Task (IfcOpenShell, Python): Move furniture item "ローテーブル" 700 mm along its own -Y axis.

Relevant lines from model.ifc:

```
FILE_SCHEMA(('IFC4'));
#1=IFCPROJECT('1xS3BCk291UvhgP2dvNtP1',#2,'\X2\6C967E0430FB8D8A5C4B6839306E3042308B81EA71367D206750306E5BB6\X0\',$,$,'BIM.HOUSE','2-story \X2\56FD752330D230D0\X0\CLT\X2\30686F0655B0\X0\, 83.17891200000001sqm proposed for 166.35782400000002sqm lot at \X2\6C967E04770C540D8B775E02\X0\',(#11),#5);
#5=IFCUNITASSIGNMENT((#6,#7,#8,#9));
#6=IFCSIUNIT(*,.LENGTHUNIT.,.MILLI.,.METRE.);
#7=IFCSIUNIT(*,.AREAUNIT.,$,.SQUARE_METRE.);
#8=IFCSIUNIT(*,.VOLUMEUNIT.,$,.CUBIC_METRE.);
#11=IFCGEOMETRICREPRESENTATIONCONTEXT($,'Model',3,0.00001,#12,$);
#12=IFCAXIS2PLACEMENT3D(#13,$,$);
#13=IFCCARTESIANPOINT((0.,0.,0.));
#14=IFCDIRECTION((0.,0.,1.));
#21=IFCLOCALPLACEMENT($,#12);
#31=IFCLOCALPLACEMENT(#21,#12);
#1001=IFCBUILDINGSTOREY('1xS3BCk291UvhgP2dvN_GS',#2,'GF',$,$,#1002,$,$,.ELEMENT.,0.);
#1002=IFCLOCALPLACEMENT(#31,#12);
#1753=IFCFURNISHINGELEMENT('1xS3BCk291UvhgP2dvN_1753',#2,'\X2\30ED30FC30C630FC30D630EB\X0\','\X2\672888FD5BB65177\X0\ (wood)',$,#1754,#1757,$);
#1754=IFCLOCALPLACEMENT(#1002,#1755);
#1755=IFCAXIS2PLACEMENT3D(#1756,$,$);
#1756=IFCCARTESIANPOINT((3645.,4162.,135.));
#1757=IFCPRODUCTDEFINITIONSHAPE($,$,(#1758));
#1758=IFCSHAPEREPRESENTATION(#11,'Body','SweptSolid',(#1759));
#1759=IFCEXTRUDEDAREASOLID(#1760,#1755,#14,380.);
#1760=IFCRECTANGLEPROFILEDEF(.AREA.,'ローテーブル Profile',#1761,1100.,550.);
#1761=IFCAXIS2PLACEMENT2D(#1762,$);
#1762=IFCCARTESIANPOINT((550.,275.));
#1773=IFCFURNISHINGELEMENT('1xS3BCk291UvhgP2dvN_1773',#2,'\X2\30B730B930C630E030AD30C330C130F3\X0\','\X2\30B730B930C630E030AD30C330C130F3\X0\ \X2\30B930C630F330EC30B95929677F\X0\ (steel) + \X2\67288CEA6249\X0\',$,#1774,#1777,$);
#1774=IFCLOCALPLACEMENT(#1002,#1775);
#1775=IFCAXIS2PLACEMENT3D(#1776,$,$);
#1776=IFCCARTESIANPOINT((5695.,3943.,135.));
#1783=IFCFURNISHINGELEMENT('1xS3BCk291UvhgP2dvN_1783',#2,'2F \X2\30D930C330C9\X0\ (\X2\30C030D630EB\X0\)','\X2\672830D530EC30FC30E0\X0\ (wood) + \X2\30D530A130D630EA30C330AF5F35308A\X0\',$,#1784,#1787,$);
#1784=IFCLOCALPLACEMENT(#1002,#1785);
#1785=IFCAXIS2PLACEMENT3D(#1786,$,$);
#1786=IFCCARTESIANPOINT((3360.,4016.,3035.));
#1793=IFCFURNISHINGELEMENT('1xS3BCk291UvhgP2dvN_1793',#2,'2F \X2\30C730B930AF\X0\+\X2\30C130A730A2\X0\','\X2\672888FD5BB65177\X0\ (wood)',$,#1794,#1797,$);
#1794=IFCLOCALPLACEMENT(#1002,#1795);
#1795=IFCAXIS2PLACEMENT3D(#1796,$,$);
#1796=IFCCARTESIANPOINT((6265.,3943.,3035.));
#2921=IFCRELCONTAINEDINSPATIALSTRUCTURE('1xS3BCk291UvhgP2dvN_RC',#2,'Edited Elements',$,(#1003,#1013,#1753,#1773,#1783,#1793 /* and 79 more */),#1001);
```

```python
import ifcopenshell
import ifcopenshell.api.geometry
import ifcopenshell.util.placement
import ifcopenshell.util.unit

model = ifcopenshell.open("model.ifc")
unit_scale = ifcopenshell.util.unit.calculate_unit_scale(model)

item = model.by_guid("1xS3BCk291UvhgP2dvN_1753")
matrix = ifcopenshell.util.placement.get_local_placement(item.ObjectPlacement)
matrix[:3, 3] -= matrix[:3, 1] * 0.7 / unit_scale
ifcopenshell.api.geometry.edit_object_placement(model, product=item, matrix=matrix, is_si=False)

print(ifcopenshell.util.placement.get_local_placement(item.ObjectPlacement).round(3) + 0.0)

model.write("model_updated.ifc")
```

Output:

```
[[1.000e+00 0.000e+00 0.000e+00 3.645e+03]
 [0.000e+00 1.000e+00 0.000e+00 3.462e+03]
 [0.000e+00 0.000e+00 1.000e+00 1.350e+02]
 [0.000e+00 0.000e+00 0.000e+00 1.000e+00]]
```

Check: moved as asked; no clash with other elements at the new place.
